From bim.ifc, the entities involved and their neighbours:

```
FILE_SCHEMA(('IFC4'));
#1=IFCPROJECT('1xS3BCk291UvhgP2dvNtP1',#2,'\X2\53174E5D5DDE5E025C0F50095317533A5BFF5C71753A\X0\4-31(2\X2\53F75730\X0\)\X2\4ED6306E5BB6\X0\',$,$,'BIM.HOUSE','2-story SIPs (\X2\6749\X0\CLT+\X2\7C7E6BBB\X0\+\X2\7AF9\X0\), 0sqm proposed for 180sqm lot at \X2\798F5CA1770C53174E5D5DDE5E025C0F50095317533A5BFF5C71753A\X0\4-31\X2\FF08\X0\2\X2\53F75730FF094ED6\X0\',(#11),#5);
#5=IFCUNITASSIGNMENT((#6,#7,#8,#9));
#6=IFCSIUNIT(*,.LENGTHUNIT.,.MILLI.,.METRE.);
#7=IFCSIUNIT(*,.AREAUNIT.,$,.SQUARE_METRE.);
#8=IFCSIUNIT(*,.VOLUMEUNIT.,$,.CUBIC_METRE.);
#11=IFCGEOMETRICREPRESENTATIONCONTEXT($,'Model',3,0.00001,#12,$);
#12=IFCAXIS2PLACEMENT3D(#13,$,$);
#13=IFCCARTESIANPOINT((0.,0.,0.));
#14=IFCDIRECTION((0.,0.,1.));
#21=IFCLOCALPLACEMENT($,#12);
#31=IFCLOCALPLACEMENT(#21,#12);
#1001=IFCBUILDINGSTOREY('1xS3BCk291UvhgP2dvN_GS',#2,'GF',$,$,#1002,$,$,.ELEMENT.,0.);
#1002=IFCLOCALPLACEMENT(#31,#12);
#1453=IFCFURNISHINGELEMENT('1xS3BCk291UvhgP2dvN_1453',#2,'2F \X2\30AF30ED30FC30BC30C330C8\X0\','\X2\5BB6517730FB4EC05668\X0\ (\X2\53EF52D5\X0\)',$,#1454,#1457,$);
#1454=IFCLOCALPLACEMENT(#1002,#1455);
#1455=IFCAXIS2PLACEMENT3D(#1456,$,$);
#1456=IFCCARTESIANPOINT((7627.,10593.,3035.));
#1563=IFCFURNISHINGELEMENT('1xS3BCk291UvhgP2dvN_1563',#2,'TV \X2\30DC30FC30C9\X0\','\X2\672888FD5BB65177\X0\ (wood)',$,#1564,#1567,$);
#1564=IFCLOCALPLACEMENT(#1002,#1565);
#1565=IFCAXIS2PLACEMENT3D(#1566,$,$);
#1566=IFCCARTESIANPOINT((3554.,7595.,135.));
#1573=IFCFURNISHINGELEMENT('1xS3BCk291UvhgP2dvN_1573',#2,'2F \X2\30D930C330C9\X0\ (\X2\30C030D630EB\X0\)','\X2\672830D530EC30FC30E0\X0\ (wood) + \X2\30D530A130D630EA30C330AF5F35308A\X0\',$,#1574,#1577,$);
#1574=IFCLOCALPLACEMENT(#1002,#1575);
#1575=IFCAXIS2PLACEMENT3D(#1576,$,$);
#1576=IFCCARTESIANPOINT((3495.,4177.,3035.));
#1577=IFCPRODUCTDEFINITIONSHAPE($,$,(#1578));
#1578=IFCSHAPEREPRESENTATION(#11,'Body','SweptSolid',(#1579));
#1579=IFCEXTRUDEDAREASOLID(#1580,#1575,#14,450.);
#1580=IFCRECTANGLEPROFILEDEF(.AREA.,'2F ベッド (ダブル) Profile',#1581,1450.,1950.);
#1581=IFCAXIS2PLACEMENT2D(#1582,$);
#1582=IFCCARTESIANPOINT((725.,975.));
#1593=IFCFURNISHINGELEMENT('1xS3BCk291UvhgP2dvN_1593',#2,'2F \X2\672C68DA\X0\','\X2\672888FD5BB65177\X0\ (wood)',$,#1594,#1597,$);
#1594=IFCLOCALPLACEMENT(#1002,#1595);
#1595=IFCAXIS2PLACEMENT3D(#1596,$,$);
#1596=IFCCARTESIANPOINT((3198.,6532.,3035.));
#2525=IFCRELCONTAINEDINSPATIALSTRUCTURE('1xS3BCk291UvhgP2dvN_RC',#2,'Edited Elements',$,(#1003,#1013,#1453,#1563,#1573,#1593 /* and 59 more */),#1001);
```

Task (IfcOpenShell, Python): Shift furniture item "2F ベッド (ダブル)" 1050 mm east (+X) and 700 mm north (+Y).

```python
import ifcopenshell
import ifcopenshell.api.geometry
import ifcopenshell.util.placement
import ifcopenshell.util.unit

model = ifcopenshell.open("bim.ifc")
unit_scale = ifcopenshell.util.unit.calculate_unit_scale(model)

item = model.by_id(1573)
matrix = ifcopenshell.util.placement.get_local_placement(item.ObjectPlacement)
matrix[0, 3] += 1.05 / unit_scale
matrix[1, 3] += 0.7 / unit_scale
ifcopenshell.api.geometry.edit_object_placement(model, product=item, matrix=matrix, is_si=False)

print(ifcopenshell.util.placement.get_local_placement(item.ObjectPlacement).round(3) + 0.0)

model.write("bim-out.ifc")
```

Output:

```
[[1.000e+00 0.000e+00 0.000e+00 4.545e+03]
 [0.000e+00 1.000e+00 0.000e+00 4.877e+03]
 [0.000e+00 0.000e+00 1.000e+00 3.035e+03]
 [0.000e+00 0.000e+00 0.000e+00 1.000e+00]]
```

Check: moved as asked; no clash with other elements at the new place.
